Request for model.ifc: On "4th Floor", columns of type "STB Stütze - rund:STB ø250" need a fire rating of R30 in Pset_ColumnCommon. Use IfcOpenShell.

First a look at what the model holds.

```python
import ifcopenshell
import ifcopenshell.util.element

model = ifcopenshell.open("model.ifc")
print(model.schema)
storey = next(s for s in model.by_type("IfcBuildingStorey") if s.Name == "4th Floor")
columns = [e for e in ifcopenshell.util.element.get_decomposition(storey) if e.is_a("IfcColumn")]
seen = {}
for e in columns:
    element_type = ifcopenshell.util.element.get_type(e)
    key = (element_type.Name if element_type != e and element_type else None, ifcopenshell.util.element.get_pset(e, "Pset_ColumnCommon", "FireRating"))
    seen[key] = seen.get(key, 0) + 1
for (name, value), count in sorted(seen.items(), key=str):
    print(count, "x", name, "|", value)
```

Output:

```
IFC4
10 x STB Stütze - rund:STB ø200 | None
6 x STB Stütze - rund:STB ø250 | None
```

```python
import ifcopenshell
import ifcopenshell.api.pset
import ifcopenshell.util.element

model = ifcopenshell.open("model.ifc")

storey = next(s for s in model.by_type("IfcBuildingStorey") if s.Name == "4th Floor")
columns = [e for e in ifcopenshell.util.element.get_decomposition(storey) if e.is_a("IfcColumn")]

count = 0
for e in columns:
    element_type = ifcopenshell.util.element.get_type(e)
    if element_type in (None, e) or element_type.Name != "STB Stütze - rund:STB ø250":
        continue
    # add_pset returns the element's existing set when there is one.
    pset = ifcopenshell.api.pset.add_pset(model, product=e, name="Pset_ColumnCommon")
    ifcopenshell.api.pset.edit_pset(model, pset=pset, properties={"FireRating": "R30"})
    count += 1

print(count, "columns updated")

model.write("model-out.ifc")
```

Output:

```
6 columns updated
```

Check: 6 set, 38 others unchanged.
